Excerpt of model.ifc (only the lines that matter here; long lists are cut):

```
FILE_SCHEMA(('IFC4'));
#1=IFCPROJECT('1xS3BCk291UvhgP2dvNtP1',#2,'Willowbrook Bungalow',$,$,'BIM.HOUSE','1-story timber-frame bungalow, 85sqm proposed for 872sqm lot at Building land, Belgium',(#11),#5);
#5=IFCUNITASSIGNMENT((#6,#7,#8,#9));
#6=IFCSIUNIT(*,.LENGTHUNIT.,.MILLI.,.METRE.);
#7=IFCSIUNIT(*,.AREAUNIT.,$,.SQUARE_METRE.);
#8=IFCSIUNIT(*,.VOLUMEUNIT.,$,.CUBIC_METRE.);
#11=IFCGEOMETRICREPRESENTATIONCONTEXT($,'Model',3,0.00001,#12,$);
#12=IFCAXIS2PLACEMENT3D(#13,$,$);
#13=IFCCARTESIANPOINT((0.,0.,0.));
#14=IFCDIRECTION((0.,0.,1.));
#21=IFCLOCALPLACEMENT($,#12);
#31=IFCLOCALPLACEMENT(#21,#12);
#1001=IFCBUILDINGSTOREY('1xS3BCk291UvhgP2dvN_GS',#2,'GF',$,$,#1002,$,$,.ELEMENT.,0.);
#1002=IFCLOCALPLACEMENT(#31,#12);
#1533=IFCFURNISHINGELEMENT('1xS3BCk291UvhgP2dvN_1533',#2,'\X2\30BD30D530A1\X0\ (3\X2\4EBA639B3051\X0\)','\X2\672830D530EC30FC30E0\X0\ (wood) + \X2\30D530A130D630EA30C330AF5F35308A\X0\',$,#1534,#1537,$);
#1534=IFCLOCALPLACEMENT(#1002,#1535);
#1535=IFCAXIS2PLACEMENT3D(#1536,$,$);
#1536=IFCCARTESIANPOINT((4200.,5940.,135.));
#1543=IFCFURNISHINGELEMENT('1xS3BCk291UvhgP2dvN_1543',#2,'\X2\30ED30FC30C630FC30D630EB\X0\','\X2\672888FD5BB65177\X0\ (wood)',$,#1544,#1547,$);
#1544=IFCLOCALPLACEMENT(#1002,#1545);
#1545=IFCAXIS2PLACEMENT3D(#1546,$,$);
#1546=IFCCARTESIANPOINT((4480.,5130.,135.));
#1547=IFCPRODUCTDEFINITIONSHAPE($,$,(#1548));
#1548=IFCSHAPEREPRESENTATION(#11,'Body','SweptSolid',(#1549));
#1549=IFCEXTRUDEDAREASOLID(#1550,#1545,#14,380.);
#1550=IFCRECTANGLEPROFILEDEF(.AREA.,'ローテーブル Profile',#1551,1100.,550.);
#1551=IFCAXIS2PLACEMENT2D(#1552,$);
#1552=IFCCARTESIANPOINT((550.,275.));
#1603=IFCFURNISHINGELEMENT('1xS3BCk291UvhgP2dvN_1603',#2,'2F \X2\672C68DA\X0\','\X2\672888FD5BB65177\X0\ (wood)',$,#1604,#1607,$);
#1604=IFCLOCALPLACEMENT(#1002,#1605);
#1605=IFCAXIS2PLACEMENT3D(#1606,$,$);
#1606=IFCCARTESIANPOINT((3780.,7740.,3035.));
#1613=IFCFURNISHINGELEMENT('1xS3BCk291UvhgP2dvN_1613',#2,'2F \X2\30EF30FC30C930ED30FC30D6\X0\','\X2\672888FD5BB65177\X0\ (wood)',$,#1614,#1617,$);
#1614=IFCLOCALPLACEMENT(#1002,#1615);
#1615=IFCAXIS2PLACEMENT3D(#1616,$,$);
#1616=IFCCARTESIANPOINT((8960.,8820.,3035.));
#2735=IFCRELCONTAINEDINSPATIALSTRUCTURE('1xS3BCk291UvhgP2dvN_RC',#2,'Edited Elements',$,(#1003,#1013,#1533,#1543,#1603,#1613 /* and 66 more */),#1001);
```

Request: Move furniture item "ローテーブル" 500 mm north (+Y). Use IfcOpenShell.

```python
import ifcopenshell
import ifcopenshell.api.geometry
import ifcopenshell.util.placement
import ifcopenshell.util.unit

model = ifcopenshell.open("model.ifc")
unit_scale = ifcopenshell.util.unit.calculate_unit_scale(model)

item = model.by_guid("1xS3BCk291UvhgP2dvN_1543")
matrix = ifcopenshell.util.placement.get_local_placement(item.ObjectPlacement)
matrix[1, 3] += 0.5 / unit_scale
ifcopenshell.api.geometry.edit_object_placement(model, product=item, matrix=matrix, is_si=False)

print(ifcopenshell.util.placement.get_local_placement(item.ObjectPlacement).round(3) + 0.0)

model.write("model_edited.ifc")
```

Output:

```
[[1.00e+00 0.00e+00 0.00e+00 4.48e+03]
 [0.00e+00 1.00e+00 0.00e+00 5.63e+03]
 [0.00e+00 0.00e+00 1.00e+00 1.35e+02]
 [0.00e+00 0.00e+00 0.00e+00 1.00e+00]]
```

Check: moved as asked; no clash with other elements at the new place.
